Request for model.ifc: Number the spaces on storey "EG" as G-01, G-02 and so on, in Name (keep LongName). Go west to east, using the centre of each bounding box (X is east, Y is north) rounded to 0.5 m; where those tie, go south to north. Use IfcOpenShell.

First a look at what the model holds.

```python
import ifcopenshell
import ifcopenshell.util.element
import ifcopenshell.util.placement

model = ifcopenshell.open("model.ifc")
print(model.schema)
storey = next(s for s in model.by_type("IfcBuildingStorey") if s.Name == "EG")
spaces = [e for e in ifcopenshell.util.element.get_decomposition(storey) if e.is_a("IfcSpace")]
for e in sorted(spaces, key=lambda e: e.id()):
    origin = ifcopenshell.util.placement.get_local_placement(e.ObjectPlacement)[:3, 3]
    print(e.id(), e.Name, e.LongName, origin.round(2) + 0.0, sep=" | ")
```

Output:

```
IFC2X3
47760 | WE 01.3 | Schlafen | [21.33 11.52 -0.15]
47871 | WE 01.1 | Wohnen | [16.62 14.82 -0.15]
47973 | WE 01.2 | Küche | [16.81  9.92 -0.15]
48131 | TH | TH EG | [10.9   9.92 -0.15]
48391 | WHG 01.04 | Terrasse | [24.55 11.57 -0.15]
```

```python
import ifcopenshell
import ifcopenshell.geom
import ifcopenshell.util.element
import ifcopenshell.util.shape

model = ifcopenshell.open("model.ifc")
settings = ifcopenshell.geom.settings()
settings.set("use-world-coords", True)


def centre(element):
    shape = ifcopenshell.geom.create_shape(settings, element)
    return ifcopenshell.util.shape.get_bbox_centroid(shape.geometry)


storey = next(s for s in model.by_type("IfcBuildingStorey") if s.Name == "EG")
spaces = [e for e in ifcopenshell.util.element.get_decomposition(storey) if e.is_a("IfcSpace")]

# Insertion points can sit at a corner or the storey origin, so sort by the geometry (in metres).
centres = {e: centre(e) for e in spaces}
spaces.sort(key=lambda e: (round(centres[e][0] / 0.5), centres[e][1]))

for i, e in enumerate(spaces, start=1):
    number = f"G-{i:02d}"
    e.Name = number
    print(e.id(), number)

model.write("model-out.ifc")
```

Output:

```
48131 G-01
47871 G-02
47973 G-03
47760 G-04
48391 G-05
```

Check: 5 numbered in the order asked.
